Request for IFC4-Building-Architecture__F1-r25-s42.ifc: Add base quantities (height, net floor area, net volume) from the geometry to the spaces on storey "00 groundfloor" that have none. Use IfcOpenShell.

First a look at what the model holds.

```python
import ifcopenshell
import ifcopenshell.util.element
import ifcopenshell.util.unit

model = ifcopenshell.open("IFC4-Building-Architecture__F1-r25-s42.ifc")
print(model.schema)
for unit_type in ("LENGTHUNIT", "AREAUNIT", "VOLUMEUNIT"):
    print(unit_type, ifcopenshell.util.unit.calculate_unit_scale(model, unit_type))
storey = next(s for s in model.by_type("IfcBuildingStorey") if s.Name == "00 groundfloor")
spaces = [e for e in ifcopenshell.util.element.get_decomposition(storey) if e.is_a("IfcSpace")]
for e in sorted(spaces, key=lambda e: e.id()):
    print(e.id(), e.is_a(), e.Name, list(ifcopenshell.util.element.get_psets(e, qtos_only=True)), sep=" | ")
```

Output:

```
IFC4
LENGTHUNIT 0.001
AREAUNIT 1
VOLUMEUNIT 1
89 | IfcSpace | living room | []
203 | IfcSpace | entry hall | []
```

```python
import ifcopenshell
import ifcopenshell.api.pset
import ifcopenshell.geom
import ifcopenshell.util.element
import ifcopenshell.util.shape
import ifcopenshell.util.unit

model = ifcopenshell.open("IFC4-Building-Architecture__F1-r25-s42.ifc")
unit_scale = ifcopenshell.util.unit.calculate_unit_scale(model)
area_scale = ifcopenshell.util.unit.calculate_unit_scale(model, "AREAUNIT")
volume_scale = ifcopenshell.util.unit.calculate_unit_scale(model, "VOLUMEUNIT")
settings = ifcopenshell.geom.settings()

storey = next(s for s in model.by_type("IfcBuildingStorey") if s.Name == "00 groundfloor")
spaces = [e for e in ifcopenshell.util.element.get_decomposition(storey) if e.is_a("IfcSpace")]

for e in sorted(spaces, key=lambda e: e.id()):
    if ifcopenshell.util.element.get_psets(e, qtos_only=True, should_inherit=False):
        continue
    # Geometry comes back in metres, in the element's own axes.
    shape = ifcopenshell.geom.create_shape(settings, e)
    values = {
        "Height": ifcopenshell.util.shape.get_z(shape.geometry) / unit_scale,
        "NetFloorArea": ifcopenshell.util.shape.get_footprint_area(shape.geometry) / area_scale,
        "NetVolume": ifcopenshell.util.shape.get_volume(shape.geometry) / volume_scale,
    }
    qto = ifcopenshell.api.pset.add_qto(model, product=e, name="Qto_SpaceBaseQuantities")
    ifcopenshell.api.pset.edit_qto(model, qto=qto, properties=values)
    print(e.id(), {k: round(v, 3) for k, v in values.items()})

model.write("IFC4-Building-Architecture__F1-r25-s42_edited.ifc")
```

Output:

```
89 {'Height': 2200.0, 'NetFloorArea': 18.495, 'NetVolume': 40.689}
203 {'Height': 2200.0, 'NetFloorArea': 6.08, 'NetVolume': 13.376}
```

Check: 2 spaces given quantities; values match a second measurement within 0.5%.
